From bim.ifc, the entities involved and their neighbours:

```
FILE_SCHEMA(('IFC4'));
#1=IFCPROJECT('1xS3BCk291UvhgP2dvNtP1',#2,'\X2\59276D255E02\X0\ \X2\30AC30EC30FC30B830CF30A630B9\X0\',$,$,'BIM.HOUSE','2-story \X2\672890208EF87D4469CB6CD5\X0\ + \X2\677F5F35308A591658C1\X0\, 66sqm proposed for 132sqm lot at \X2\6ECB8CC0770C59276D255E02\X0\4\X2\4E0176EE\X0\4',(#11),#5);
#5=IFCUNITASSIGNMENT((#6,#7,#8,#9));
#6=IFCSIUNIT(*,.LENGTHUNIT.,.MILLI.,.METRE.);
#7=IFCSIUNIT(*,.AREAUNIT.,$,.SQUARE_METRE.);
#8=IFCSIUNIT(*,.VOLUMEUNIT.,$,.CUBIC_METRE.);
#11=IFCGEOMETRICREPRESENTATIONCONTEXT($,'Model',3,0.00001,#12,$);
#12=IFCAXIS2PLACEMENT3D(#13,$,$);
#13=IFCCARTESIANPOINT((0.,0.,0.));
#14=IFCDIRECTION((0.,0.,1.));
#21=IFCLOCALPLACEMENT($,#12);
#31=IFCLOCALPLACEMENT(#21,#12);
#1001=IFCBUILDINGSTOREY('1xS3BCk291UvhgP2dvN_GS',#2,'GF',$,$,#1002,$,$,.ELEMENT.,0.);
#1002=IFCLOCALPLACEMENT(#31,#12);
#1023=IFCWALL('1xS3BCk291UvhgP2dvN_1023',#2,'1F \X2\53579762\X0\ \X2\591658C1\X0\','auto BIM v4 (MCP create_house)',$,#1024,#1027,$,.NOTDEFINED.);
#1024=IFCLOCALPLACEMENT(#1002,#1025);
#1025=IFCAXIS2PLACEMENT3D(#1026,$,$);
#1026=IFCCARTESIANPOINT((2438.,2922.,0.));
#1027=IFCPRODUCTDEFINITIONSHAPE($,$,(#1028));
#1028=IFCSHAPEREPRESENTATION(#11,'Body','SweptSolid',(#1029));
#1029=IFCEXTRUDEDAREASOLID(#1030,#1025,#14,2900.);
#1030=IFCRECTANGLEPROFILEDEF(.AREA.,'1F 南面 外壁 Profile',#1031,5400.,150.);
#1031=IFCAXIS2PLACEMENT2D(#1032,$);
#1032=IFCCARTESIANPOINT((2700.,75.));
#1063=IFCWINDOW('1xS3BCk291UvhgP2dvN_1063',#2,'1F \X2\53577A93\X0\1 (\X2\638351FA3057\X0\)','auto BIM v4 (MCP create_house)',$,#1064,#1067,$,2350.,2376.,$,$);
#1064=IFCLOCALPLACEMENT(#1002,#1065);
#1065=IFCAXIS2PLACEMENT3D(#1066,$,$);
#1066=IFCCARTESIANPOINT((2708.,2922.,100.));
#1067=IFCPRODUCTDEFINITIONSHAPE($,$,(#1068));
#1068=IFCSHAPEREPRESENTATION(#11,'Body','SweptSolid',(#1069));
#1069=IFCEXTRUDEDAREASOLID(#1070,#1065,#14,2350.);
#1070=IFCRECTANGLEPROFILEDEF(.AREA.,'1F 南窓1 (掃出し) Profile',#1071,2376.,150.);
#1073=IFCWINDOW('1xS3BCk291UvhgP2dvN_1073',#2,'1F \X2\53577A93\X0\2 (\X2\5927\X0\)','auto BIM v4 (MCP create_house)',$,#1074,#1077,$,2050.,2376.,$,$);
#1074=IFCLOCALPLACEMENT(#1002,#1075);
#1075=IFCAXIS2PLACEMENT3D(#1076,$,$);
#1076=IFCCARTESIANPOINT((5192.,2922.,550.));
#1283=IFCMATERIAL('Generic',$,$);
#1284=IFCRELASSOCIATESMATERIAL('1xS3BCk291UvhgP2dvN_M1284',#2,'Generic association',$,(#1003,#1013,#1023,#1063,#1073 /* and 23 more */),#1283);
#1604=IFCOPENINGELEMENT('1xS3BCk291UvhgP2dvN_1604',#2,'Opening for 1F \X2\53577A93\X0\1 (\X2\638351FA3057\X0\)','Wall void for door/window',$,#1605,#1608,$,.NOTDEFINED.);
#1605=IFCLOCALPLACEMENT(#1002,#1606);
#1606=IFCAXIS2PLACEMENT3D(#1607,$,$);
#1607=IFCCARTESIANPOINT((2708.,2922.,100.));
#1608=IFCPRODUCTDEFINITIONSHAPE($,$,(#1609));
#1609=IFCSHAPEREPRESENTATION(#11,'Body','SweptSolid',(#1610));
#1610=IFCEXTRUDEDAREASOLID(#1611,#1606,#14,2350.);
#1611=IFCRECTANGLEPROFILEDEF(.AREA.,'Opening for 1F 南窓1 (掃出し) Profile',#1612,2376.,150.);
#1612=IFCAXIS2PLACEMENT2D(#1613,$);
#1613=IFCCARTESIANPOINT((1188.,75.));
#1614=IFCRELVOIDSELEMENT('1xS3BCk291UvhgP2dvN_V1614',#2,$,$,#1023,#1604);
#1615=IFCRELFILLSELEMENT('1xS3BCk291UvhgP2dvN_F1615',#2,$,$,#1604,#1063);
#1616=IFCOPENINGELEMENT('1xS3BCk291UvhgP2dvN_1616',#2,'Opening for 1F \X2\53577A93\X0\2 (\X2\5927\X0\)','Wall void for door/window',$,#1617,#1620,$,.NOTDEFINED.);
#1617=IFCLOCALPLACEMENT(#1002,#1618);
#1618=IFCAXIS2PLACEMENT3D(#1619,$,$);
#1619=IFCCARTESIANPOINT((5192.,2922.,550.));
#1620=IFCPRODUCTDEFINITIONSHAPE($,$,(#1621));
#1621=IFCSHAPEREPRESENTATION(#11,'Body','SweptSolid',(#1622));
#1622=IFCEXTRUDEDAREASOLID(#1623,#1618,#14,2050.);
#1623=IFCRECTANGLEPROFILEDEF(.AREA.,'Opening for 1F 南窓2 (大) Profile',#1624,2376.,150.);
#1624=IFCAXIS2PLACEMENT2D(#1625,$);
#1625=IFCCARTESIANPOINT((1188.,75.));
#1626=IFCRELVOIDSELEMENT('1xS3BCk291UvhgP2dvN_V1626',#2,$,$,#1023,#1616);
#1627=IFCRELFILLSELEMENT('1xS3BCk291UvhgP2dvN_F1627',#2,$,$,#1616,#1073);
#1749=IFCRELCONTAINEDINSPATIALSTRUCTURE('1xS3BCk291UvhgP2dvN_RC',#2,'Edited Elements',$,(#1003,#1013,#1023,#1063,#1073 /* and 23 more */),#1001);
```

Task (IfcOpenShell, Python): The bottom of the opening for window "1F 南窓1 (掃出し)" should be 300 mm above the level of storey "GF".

```python
import numpy as np
import ifcopenshell
import ifcopenshell.api.geometry
import ifcopenshell.geom
import ifcopenshell.util.element
import ifcopenshell.util.placement
import ifcopenshell.util.shape
import ifcopenshell.util.unit

model = ifcopenshell.open("bim.ifc")
unit_scale = ifcopenshell.util.unit.calculate_unit_scale(model)

window = model.by_id(1063)
opening = window.FillsVoids[0].RelatingOpeningElement
storey = ifcopenshell.util.element.get_container(window, ifc_class="IfcBuildingStorey")
level = ifcopenshell.util.placement.get_local_placement(storey.ObjectPlacement)[2, 3]

# The opening's origin need not be at the sill, so measure its lowest point.
shape = ifcopenshell.geom.create_shape(ifcopenshell.geom.settings(), opening)
bottom = ifcopenshell.util.shape.get_shape_bottom_elevation(shape, shape.geometry) / unit_scale
dz = level + 0.3 / unit_scale - bottom

shift = np.array([0.0, 0.0, dz])
# The window is not placed relative to its opening, so move both.
for product in (opening, window):
    matrix = ifcopenshell.util.placement.get_local_placement(product.ObjectPlacement)
    matrix[:3, 3] += shift
    ifcopenshell.api.geometry.edit_object_placement(model, product=product, matrix=matrix, is_si=False)

print(f"moved by {dz * unit_scale:+.3f} m")

model.write("bim-out.ifc")
```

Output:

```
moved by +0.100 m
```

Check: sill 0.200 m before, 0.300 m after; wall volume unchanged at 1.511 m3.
